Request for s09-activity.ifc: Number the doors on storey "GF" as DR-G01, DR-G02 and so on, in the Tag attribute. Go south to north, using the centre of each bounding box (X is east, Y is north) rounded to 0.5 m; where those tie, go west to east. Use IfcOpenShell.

First a look at what the model holds.

```python
import ifcopenshell
import ifcopenshell.util.element
import ifcopenshell.util.placement

model = ifcopenshell.open("s09-activity.ifc")
print(model.schema)
storey = next(s for s in model.by_type("IfcBuildingStorey") if s.Name == "GF")
doors = [e for e in ifcopenshell.util.element.get_decomposition(storey) if e.is_a("IfcDoor")]
for e in sorted(doors, key=lambda e: e.id()):
    origin = ifcopenshell.util.placement.get_local_placement(e.ObjectPlacement)[:3, 3]
    print(e.id(), e.Tag, e.Name, origin.round(2) + 0.0, sep=" | ")
```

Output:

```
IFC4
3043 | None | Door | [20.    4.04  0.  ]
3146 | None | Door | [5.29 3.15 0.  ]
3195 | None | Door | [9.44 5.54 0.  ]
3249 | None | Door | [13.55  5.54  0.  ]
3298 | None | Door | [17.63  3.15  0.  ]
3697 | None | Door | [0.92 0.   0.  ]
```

```python
import ifcopenshell
import ifcopenshell.geom
import ifcopenshell.util.element
import ifcopenshell.util.shape

model = ifcopenshell.open("s09-activity.ifc")
settings = ifcopenshell.geom.settings()
settings.set("use-world-coords", True)


def centre(element):
    shape = ifcopenshell.geom.create_shape(settings, element)
    return ifcopenshell.util.shape.get_bbox_centroid(shape.geometry)


storey = next(s for s in model.by_type("IfcBuildingStorey") if s.Name == "GF")
doors = [e for e in ifcopenshell.util.element.get_decomposition(storey) if e.is_a("IfcDoor")]

# Insertion points can sit at a corner or the storey origin, so sort by the geometry (in metres).
centres = {e: centre(e) for e in doors}
doors.sort(key=lambda e: (round(centres[e][1] / 0.5), centres[e][0]))

for i, e in enumerate(doors, start=1):
    number = f"DR-G{i:02d}"
    e.Tag = number
    print(e.id(), number)

model.write("s09-activity_v2.ifc")
```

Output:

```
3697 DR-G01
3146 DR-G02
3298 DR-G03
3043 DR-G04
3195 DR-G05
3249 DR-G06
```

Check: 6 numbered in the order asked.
